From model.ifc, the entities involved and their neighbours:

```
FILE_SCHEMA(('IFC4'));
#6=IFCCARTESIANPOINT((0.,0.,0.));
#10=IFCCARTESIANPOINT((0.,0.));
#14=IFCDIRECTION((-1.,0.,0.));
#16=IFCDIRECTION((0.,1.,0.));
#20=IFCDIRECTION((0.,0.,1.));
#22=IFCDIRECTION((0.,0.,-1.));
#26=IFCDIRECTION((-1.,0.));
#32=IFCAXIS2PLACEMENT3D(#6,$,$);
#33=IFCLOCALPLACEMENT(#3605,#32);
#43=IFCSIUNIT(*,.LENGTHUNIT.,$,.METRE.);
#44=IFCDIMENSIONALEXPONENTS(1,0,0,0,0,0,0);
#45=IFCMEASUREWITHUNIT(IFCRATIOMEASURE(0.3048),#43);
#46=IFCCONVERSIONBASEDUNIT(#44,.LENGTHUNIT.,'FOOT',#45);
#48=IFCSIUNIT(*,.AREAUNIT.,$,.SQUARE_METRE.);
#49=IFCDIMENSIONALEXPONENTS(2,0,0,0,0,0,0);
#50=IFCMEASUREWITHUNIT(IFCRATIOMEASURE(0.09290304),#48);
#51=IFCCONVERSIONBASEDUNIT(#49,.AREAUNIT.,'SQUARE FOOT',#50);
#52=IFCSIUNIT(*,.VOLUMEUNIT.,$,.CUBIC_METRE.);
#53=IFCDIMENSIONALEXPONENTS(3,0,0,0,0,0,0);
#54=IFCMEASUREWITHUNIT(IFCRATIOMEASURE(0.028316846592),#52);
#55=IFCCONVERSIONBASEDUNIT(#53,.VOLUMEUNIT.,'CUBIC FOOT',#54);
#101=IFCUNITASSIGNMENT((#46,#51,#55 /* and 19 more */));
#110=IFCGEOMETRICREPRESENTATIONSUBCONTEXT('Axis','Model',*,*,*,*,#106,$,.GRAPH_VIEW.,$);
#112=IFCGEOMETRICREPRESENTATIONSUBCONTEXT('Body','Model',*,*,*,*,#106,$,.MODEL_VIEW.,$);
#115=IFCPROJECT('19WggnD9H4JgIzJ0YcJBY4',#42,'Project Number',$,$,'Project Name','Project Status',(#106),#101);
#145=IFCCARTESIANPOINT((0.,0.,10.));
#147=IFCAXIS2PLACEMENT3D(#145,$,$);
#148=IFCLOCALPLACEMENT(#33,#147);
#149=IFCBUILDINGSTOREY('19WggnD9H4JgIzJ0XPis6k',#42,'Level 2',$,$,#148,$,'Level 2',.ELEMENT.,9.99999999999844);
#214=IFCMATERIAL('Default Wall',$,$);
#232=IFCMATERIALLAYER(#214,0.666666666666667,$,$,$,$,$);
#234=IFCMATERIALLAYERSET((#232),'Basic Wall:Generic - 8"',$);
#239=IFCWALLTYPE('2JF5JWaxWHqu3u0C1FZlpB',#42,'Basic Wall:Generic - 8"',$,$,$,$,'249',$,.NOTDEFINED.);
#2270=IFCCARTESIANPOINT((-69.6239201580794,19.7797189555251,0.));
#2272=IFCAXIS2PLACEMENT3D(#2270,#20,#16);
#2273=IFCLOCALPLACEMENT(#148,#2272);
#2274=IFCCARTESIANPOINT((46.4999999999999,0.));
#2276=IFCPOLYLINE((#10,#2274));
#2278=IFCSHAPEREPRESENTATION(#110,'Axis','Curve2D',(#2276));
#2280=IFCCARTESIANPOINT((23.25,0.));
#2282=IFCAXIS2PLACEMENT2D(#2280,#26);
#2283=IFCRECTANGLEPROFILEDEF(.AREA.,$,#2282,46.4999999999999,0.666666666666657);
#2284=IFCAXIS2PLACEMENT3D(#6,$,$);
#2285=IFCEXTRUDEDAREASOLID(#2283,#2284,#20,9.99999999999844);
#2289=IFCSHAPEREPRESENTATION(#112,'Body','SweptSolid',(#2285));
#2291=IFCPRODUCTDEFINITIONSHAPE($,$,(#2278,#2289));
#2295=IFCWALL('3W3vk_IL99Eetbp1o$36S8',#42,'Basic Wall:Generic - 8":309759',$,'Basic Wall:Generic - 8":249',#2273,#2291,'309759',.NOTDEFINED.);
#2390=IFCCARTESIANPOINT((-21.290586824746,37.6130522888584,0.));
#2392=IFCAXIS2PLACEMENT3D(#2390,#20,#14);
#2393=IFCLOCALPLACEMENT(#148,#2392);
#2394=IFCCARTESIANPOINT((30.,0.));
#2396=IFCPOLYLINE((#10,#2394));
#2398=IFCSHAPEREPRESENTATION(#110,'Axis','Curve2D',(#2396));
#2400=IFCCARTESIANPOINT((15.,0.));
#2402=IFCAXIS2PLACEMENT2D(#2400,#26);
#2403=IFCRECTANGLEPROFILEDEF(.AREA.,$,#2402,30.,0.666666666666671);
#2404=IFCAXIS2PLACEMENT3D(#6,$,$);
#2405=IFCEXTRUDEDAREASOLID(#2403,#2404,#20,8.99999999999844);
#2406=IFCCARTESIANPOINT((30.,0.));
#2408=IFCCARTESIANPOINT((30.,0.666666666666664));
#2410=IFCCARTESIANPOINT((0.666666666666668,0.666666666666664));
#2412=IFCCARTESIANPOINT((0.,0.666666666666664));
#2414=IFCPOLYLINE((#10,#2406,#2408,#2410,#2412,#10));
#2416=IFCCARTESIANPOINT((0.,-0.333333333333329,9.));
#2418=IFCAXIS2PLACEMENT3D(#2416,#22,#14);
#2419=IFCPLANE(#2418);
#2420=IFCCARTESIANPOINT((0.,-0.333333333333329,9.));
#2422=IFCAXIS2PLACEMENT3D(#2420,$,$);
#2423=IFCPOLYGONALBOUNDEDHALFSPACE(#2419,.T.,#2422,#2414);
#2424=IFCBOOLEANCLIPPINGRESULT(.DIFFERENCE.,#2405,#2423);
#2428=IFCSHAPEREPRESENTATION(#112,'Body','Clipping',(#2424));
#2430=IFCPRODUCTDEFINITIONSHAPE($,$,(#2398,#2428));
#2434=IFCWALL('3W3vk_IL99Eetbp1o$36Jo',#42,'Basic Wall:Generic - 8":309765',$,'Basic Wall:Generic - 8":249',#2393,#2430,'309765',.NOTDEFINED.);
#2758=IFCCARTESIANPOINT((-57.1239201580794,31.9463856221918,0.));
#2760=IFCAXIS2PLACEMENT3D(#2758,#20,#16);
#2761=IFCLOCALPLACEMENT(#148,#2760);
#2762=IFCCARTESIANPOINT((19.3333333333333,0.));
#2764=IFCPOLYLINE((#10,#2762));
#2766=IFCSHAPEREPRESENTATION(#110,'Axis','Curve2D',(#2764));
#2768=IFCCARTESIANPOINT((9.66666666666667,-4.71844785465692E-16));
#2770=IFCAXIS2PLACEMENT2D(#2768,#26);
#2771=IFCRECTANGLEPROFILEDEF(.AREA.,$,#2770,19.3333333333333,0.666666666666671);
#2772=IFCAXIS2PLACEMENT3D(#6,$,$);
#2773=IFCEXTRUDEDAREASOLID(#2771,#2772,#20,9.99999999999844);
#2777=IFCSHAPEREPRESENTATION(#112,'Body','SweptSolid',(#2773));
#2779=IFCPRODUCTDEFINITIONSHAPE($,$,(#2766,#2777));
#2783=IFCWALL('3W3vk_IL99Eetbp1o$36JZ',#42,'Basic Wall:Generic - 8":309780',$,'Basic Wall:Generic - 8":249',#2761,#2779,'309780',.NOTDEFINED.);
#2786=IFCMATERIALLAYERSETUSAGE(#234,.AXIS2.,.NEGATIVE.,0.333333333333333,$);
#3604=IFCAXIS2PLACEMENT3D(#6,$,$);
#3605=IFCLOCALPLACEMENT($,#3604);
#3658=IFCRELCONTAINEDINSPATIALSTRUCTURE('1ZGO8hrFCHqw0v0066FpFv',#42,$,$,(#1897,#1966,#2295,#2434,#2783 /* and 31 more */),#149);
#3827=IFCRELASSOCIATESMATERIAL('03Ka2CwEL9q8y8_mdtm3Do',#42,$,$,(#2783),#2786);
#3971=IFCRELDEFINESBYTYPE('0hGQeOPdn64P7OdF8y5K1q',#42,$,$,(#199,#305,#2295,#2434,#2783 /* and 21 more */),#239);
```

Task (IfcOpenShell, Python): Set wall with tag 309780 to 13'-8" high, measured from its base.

```python
import ifcopenshell
import ifcopenshell.geom
import ifcopenshell.util.representation
import ifcopenshell.util.shape
import ifcopenshell.util.unit

model = ifcopenshell.open("model.ifc")
unit_scale = ifcopenshell.util.unit.calculate_unit_scale(model)
settings = ifcopenshell.geom.settings()


def volume(element):
    """Net volume in cubic metres, openings subtracted."""
    shape = ifcopenshell.geom.create_shape(settings, element)
    return ifcopenshell.util.shape.get_volume(shape.geometry)


wall = model.by_guid("3W3vk_IL99Eetbp1o$36JZ")
before = volume(wall)

body = ifcopenshell.util.representation.get_representation(wall, "Model", "Body")
solid = body.Items[0]
old_height = solid.Depth
solid.Depth = 164 * 0.0254 / unit_scale
after = volume(wall)

print(f"height {old_height:g} -> {solid.Depth:g}, volume {before:.3f} -> {after:.3f} m3")

model.write("model_edited.ifc")
```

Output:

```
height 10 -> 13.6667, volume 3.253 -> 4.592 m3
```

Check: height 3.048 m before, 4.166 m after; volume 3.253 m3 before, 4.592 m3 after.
